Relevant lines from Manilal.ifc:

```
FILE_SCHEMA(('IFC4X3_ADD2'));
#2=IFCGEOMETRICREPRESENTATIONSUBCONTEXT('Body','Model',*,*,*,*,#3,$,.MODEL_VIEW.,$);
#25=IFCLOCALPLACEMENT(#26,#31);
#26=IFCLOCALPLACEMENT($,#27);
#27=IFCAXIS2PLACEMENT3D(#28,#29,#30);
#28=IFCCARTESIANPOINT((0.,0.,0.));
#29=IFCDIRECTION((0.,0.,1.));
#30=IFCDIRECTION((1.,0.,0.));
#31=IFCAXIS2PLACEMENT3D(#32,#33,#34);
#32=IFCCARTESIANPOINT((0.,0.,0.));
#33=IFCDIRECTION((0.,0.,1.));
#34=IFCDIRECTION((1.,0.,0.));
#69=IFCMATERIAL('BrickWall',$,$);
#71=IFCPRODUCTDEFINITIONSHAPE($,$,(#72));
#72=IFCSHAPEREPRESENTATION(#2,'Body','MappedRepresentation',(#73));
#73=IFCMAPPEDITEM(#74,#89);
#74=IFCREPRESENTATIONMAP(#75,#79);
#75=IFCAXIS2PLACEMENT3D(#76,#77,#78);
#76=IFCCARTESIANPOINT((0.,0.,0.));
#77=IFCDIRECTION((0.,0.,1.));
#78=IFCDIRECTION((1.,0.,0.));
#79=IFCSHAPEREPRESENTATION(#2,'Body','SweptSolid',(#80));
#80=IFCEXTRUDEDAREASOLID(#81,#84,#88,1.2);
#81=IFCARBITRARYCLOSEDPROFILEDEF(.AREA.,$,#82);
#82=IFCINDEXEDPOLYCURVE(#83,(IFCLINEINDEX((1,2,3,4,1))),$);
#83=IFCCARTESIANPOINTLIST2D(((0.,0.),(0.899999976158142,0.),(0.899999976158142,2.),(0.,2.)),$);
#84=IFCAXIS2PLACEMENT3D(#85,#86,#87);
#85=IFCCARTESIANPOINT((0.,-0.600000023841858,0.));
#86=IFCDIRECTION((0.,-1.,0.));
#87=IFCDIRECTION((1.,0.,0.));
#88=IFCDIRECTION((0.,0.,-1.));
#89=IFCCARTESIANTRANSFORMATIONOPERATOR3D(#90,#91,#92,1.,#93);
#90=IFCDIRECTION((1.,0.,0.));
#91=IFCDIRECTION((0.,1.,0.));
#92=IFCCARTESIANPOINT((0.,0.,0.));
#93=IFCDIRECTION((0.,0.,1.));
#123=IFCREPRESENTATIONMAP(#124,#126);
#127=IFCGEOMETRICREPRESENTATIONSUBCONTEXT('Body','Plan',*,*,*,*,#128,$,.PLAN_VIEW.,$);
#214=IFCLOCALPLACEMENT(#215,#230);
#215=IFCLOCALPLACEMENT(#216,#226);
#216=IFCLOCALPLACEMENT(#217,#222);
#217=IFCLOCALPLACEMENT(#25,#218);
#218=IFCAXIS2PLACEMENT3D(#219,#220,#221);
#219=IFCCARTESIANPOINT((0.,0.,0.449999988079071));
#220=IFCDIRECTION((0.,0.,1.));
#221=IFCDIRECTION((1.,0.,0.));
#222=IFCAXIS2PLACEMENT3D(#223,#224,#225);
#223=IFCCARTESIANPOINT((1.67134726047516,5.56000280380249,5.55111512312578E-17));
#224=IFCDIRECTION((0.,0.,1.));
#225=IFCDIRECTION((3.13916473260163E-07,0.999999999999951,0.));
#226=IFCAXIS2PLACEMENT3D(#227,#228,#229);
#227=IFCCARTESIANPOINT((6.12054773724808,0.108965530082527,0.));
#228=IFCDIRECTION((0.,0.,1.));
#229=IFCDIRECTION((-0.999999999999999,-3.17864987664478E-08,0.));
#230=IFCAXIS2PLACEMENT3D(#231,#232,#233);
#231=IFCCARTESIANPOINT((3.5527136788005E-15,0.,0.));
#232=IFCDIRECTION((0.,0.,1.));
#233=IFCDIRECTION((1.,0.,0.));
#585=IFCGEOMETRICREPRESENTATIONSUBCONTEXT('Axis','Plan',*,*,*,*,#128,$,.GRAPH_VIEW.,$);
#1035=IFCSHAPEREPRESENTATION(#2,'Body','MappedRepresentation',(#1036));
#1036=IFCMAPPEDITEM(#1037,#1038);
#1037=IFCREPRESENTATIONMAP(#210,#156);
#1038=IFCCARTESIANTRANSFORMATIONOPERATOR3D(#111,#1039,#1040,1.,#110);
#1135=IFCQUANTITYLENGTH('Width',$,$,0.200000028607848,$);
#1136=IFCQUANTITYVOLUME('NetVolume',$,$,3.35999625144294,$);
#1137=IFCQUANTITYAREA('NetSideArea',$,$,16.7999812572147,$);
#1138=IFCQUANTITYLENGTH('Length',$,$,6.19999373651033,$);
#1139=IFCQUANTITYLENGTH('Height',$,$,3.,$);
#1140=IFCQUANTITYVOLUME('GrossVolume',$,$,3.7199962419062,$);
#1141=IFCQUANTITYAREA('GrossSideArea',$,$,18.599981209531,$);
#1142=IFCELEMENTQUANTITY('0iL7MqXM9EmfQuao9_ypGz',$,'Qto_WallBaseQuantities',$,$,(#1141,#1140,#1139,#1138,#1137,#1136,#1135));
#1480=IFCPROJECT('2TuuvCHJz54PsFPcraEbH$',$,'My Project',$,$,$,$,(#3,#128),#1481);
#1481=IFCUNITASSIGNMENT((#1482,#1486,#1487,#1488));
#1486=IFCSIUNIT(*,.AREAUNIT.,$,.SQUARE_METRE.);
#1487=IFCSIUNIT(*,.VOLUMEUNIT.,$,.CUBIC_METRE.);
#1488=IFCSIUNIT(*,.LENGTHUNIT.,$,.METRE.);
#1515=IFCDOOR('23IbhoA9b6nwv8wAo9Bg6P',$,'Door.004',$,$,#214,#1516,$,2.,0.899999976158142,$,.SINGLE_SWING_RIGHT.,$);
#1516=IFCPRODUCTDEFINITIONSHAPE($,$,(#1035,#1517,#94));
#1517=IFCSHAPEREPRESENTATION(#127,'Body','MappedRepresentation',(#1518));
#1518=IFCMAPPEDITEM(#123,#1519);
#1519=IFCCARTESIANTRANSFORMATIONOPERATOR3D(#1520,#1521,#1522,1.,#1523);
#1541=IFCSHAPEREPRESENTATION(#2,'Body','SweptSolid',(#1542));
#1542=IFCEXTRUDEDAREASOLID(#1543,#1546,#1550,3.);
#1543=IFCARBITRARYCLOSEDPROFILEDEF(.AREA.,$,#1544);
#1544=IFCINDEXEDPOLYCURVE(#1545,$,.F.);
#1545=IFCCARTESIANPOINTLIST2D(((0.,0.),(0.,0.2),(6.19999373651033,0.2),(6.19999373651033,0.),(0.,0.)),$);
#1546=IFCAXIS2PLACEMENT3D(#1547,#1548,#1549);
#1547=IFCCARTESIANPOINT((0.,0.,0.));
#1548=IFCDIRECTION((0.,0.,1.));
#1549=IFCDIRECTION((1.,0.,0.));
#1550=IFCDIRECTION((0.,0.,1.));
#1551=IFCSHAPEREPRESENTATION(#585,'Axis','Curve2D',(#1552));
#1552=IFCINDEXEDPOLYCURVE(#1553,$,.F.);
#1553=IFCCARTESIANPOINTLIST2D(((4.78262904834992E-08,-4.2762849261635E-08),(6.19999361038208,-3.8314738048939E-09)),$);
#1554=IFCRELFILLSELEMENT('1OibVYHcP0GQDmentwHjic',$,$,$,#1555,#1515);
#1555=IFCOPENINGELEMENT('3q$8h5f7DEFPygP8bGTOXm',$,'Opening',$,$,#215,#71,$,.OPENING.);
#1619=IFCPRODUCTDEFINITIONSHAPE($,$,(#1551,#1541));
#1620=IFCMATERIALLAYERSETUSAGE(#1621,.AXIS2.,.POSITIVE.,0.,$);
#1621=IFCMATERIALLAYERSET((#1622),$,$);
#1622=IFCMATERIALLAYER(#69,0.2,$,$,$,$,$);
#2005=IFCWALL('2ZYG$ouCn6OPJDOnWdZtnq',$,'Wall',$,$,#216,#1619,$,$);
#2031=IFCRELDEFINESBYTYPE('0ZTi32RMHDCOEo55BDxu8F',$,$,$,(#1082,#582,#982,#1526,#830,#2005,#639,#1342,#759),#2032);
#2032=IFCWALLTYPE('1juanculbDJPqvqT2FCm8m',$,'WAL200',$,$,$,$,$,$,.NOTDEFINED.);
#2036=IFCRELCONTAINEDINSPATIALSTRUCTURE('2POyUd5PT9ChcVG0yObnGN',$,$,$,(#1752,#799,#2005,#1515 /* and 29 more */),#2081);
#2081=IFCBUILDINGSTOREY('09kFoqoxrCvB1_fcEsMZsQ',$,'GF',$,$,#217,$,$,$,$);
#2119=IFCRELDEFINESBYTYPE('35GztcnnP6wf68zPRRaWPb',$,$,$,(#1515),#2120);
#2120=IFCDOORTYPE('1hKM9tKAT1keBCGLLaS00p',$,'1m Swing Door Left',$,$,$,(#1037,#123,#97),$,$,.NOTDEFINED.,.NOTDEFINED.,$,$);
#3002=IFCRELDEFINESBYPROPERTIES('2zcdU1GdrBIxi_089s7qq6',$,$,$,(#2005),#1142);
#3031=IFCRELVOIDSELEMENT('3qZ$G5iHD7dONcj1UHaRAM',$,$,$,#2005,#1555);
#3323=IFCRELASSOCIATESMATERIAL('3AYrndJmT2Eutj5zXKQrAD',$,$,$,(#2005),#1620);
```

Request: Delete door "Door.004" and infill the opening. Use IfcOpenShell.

```python
import ifcopenshell
import ifcopenshell.api.feature
import ifcopenshell.api.pset
import ifcopenshell.api.root
import ifcopenshell.geom
import ifcopenshell.util.element
import ifcopenshell.util.shape
import ifcopenshell.util.unit

model = ifcopenshell.open("Manilal.ifc")
area_scale = ifcopenshell.util.unit.calculate_unit_scale(model, "AREAUNIT")
volume_scale = ifcopenshell.util.unit.calculate_unit_scale(model, "VOLUMEUNIT")
settings = ifcopenshell.geom.settings()


def volume(element):
    """Net volume in cubic metres, openings subtracted."""
    shape = ifcopenshell.geom.create_shape(settings, element)
    return ifcopenshell.util.shape.get_volume(shape.geometry)


door = model.by_guid("23IbhoA9b6nwv8wAo9Bg6P")
opening = door.FillsVoids[0].RelatingOpeningElement
wall = opening.VoidsElements[0].RelatingBuildingElement
before = volume(wall)

ifcopenshell.api.root.remove_product(model, product=door)
ifcopenshell.api.feature.remove_feature(model, feature=opening)

after = volume(wall)
thickness = 0.2  # wall thickness in metres

# Update the wall's stored quantities.
qto = model.by_id(ifcopenshell.util.element.get_pset(wall, "Qto_WallBaseQuantities", should_inherit=False)["id"])
ifcopenshell.api.pset.edit_qto(model, qto=qto, properties={
    "NetSideArea": after / thickness / area_scale,
    "NetVolume": after / volume_scale,
})

print(f"wall volume {before:.3f} -> {after:.3f} m3")

model.write("Manilal-out.ifc")
```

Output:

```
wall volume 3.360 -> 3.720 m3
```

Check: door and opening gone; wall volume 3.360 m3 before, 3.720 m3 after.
